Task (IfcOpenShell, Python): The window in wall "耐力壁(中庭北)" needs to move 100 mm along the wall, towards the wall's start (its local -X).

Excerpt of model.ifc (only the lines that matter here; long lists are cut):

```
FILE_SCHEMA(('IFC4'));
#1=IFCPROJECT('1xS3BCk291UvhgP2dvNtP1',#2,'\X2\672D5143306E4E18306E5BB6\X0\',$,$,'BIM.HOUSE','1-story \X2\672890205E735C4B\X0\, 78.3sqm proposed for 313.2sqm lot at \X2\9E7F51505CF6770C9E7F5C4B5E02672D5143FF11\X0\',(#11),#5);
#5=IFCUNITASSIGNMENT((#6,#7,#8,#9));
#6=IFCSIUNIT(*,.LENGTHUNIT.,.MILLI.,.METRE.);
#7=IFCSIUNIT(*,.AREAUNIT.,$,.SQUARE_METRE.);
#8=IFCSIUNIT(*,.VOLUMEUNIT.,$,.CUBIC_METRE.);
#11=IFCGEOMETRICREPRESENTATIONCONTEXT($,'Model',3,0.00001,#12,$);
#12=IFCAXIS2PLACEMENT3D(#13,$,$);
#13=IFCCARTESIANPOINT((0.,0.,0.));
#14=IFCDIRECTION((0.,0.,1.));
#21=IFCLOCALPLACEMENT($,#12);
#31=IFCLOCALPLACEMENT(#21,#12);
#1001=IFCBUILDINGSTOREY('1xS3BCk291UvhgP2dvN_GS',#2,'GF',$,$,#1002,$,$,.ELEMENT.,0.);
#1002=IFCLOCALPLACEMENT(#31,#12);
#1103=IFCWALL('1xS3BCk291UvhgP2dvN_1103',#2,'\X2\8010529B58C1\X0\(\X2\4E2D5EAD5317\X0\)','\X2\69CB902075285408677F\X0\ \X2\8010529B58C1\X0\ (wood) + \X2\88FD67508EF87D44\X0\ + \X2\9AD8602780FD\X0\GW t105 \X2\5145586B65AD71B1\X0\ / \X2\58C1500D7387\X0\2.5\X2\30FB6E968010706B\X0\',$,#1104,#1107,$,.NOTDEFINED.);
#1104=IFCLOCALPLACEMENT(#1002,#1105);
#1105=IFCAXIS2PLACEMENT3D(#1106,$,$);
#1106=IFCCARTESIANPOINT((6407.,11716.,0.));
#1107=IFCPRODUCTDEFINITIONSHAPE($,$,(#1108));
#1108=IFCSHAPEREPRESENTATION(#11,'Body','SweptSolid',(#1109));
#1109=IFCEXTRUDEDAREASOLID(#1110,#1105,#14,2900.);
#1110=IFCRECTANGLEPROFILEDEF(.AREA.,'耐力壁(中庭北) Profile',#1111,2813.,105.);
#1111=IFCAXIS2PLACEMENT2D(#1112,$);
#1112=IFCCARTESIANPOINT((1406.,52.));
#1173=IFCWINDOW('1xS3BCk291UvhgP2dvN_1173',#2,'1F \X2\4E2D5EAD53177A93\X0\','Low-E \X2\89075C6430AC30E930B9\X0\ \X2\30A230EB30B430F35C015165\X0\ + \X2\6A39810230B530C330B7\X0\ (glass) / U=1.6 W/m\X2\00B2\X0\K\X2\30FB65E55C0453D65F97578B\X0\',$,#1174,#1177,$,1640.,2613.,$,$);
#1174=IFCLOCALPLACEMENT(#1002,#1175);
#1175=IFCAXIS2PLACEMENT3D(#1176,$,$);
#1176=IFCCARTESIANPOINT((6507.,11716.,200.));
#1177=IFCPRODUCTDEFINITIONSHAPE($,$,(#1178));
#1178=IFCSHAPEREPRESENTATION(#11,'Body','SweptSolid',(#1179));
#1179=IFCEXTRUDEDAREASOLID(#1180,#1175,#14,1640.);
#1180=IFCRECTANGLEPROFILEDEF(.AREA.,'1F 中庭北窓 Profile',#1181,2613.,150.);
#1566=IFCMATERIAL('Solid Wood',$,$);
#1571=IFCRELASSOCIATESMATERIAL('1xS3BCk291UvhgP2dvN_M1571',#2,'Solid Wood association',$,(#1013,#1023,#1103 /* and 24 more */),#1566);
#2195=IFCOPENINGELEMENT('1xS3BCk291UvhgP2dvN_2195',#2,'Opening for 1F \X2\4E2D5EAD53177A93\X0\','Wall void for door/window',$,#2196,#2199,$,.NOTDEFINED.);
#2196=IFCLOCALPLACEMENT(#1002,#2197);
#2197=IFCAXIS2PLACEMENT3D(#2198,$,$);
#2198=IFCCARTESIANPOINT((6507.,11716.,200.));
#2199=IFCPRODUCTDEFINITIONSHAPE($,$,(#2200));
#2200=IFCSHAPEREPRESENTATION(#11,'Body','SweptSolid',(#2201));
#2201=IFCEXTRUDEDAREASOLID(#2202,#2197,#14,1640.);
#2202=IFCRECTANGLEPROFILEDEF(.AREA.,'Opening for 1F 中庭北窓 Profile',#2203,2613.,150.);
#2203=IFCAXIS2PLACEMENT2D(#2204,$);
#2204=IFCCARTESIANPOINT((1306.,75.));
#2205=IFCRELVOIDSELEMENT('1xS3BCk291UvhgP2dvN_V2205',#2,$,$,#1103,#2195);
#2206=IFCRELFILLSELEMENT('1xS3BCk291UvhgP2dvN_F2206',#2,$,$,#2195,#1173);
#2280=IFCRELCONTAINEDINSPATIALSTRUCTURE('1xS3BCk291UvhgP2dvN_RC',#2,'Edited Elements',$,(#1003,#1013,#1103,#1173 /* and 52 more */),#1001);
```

```python
import ifcopenshell
import ifcopenshell.api.geometry
import ifcopenshell.util.placement

model = ifcopenshell.open("model.ifc")

window = model.by_guid("1xS3BCk291UvhgP2dvN_1173")
opening = window.FillsVoids[0].RelatingOpeningElement
wall = opening.VoidsElements[0].RelatingBuildingElement

wall_matrix = ifcopenshell.util.placement.get_local_placement(wall.ObjectPlacement)
shift = wall_matrix[:3, 0] * -100.0
before = ifcopenshell.util.placement.get_local_placement(window.ObjectPlacement)[:3, 3].copy()

# The window is not placed relative to its opening, so move both.
for product in (opening, window):
    matrix = ifcopenshell.util.placement.get_local_placement(product.ObjectPlacement)
    matrix[:3, 3] += shift
    ifcopenshell.api.geometry.edit_object_placement(model, product=product, matrix=matrix, is_si=False)

after = ifcopenshell.util.placement.get_local_placement(window.ObjectPlacement)[:3, 3]
print("window moved by", (after - before).round(3) + 0.0)

model.write("model_updated.ifc")
```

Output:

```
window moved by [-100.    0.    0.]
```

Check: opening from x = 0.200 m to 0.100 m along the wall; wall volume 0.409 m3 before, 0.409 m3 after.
